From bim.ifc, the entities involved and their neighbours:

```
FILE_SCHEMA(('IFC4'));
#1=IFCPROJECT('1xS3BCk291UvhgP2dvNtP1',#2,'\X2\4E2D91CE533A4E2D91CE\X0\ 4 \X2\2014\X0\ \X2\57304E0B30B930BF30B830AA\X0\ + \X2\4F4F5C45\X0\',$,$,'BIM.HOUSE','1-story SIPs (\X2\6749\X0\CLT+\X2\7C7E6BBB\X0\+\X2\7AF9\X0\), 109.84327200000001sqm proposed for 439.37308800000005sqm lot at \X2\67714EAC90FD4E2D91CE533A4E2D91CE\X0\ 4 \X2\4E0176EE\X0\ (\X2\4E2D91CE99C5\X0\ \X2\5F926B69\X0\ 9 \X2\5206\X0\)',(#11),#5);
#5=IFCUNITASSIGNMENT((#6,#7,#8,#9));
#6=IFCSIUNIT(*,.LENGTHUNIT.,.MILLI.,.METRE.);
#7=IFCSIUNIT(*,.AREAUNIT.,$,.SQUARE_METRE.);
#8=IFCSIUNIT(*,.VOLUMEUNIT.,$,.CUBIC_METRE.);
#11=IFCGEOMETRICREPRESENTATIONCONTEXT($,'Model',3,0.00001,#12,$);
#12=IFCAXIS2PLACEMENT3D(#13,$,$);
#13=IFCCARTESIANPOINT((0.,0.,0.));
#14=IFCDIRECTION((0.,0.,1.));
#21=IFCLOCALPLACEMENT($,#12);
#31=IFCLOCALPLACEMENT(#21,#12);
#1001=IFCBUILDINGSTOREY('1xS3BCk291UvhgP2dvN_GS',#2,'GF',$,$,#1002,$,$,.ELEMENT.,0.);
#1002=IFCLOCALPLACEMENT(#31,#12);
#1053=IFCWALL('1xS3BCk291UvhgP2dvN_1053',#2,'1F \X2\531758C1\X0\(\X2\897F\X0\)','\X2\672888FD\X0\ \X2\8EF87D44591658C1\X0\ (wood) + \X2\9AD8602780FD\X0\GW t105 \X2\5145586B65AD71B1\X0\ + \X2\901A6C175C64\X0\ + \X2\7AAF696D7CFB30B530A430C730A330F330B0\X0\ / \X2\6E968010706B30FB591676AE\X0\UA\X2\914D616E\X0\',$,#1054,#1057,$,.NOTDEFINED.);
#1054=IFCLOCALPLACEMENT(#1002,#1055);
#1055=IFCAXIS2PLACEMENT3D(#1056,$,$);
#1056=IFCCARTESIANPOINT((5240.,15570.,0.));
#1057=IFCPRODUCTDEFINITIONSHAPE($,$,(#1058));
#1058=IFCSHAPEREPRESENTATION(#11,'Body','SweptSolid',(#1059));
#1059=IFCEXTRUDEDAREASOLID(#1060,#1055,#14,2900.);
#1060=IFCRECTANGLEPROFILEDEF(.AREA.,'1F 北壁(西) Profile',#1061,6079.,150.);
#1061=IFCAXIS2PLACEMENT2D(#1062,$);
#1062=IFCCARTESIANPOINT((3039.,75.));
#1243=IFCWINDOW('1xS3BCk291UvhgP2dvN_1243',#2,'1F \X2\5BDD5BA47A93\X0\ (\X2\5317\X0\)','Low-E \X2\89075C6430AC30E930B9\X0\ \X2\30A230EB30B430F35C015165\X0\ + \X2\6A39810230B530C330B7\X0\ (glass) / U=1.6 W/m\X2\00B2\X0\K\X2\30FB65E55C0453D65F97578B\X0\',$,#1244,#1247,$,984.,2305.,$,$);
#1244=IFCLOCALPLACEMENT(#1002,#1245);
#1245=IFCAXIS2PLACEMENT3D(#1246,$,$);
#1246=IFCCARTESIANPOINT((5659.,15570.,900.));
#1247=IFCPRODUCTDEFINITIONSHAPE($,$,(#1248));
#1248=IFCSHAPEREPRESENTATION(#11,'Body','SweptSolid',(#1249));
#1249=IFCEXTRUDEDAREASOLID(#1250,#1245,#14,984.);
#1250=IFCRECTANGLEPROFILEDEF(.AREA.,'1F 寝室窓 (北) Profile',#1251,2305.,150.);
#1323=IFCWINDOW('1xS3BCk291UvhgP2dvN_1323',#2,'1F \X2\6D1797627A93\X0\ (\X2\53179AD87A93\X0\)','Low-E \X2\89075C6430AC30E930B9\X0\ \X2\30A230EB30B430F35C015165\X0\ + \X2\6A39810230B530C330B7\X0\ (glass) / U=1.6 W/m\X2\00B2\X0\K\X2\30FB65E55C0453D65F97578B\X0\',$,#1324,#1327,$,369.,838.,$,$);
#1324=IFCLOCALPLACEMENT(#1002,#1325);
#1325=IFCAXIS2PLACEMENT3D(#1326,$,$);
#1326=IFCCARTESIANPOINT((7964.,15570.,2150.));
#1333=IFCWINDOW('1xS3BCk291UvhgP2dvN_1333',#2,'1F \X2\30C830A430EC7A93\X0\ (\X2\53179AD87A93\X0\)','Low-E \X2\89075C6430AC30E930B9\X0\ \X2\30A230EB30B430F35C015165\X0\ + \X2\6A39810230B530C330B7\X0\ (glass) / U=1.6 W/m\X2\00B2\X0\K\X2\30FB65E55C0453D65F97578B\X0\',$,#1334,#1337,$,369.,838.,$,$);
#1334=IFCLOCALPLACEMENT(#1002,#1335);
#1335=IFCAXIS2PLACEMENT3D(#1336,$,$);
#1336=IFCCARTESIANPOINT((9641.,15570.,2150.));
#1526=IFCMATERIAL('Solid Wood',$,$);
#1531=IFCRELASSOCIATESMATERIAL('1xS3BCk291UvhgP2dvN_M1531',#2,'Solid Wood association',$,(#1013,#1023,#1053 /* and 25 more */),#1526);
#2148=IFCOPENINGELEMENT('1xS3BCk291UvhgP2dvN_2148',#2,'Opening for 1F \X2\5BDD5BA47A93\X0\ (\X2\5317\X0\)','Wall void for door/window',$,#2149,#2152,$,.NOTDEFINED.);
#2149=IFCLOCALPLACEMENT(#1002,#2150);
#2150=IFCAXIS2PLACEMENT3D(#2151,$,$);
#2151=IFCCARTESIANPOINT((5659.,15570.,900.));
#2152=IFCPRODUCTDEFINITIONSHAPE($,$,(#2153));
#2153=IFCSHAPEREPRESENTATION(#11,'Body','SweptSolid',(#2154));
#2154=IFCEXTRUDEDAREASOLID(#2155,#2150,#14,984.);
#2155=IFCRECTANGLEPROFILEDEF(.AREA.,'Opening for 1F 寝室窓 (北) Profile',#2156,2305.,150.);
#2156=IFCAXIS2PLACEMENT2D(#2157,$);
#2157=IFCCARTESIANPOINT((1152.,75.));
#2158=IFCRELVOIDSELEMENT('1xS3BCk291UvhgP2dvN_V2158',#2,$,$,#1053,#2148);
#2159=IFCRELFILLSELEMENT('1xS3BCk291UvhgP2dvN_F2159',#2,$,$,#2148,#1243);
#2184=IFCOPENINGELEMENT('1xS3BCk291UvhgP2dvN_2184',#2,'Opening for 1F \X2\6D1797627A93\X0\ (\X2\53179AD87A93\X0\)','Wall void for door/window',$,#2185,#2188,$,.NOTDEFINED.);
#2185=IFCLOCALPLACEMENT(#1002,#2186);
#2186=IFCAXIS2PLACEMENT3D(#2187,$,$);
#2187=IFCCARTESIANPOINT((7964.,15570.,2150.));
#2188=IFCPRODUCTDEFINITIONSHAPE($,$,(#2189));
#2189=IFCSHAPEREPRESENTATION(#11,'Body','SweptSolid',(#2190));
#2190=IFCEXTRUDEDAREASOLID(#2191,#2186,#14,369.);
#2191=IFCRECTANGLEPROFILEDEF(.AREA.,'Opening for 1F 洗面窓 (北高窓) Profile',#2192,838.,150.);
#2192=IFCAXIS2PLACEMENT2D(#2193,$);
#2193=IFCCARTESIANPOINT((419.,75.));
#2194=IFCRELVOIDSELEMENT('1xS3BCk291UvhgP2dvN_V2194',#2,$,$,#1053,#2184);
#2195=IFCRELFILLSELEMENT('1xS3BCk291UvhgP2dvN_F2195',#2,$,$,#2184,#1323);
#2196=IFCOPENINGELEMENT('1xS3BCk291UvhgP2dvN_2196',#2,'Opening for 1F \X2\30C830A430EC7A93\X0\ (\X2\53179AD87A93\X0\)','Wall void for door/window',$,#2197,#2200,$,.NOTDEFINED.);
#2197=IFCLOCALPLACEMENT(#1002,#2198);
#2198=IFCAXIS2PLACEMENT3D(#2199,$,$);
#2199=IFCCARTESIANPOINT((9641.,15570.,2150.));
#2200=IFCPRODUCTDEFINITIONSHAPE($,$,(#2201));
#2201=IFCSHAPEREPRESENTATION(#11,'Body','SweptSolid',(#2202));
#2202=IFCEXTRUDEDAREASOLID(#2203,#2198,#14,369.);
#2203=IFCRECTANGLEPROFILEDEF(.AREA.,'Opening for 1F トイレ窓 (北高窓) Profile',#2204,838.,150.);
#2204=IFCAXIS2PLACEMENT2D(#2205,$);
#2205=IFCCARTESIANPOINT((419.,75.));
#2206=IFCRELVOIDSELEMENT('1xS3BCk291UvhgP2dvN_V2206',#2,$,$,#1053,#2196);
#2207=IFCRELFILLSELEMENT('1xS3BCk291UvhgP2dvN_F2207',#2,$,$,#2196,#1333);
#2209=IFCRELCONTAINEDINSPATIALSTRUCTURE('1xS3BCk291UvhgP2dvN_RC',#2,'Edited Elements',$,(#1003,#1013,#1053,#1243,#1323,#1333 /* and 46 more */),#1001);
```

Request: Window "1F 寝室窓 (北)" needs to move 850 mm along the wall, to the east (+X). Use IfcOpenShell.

```python
import ifcopenshell
import ifcopenshell.api.geometry
import ifcopenshell.util.placement

model = ifcopenshell.open("bim.ifc")

window = model.by_guid("1xS3BCk291UvhgP2dvN_1243")
opening = window.FillsVoids[0].RelatingOpeningElement
wall = opening.VoidsElements[0].RelatingBuildingElement

wall_matrix = ifcopenshell.util.placement.get_local_placement(wall.ObjectPlacement)
shift = wall_matrix[:3, 0] * 850.0
before = ifcopenshell.util.placement.get_local_placement(window.ObjectPlacement)[:3, 3].copy()

# The window is not placed relative to its opening, so move both.
for product in (opening, window):
    matrix = ifcopenshell.util.placement.get_local_placement(product.ObjectPlacement)
    matrix[:3, 3] += shift
    ifcopenshell.api.geometry.edit_object_placement(model, product=product, matrix=matrix, is_si=False)

after = ifcopenshell.util.placement.get_local_placement(window.ObjectPlacement)[:3, 3]
print("window moved by", (after - before).round(3) + 0.0)

model.write("bim_v2.ifc")
```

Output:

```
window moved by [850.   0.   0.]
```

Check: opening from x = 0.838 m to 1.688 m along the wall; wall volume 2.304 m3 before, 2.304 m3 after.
